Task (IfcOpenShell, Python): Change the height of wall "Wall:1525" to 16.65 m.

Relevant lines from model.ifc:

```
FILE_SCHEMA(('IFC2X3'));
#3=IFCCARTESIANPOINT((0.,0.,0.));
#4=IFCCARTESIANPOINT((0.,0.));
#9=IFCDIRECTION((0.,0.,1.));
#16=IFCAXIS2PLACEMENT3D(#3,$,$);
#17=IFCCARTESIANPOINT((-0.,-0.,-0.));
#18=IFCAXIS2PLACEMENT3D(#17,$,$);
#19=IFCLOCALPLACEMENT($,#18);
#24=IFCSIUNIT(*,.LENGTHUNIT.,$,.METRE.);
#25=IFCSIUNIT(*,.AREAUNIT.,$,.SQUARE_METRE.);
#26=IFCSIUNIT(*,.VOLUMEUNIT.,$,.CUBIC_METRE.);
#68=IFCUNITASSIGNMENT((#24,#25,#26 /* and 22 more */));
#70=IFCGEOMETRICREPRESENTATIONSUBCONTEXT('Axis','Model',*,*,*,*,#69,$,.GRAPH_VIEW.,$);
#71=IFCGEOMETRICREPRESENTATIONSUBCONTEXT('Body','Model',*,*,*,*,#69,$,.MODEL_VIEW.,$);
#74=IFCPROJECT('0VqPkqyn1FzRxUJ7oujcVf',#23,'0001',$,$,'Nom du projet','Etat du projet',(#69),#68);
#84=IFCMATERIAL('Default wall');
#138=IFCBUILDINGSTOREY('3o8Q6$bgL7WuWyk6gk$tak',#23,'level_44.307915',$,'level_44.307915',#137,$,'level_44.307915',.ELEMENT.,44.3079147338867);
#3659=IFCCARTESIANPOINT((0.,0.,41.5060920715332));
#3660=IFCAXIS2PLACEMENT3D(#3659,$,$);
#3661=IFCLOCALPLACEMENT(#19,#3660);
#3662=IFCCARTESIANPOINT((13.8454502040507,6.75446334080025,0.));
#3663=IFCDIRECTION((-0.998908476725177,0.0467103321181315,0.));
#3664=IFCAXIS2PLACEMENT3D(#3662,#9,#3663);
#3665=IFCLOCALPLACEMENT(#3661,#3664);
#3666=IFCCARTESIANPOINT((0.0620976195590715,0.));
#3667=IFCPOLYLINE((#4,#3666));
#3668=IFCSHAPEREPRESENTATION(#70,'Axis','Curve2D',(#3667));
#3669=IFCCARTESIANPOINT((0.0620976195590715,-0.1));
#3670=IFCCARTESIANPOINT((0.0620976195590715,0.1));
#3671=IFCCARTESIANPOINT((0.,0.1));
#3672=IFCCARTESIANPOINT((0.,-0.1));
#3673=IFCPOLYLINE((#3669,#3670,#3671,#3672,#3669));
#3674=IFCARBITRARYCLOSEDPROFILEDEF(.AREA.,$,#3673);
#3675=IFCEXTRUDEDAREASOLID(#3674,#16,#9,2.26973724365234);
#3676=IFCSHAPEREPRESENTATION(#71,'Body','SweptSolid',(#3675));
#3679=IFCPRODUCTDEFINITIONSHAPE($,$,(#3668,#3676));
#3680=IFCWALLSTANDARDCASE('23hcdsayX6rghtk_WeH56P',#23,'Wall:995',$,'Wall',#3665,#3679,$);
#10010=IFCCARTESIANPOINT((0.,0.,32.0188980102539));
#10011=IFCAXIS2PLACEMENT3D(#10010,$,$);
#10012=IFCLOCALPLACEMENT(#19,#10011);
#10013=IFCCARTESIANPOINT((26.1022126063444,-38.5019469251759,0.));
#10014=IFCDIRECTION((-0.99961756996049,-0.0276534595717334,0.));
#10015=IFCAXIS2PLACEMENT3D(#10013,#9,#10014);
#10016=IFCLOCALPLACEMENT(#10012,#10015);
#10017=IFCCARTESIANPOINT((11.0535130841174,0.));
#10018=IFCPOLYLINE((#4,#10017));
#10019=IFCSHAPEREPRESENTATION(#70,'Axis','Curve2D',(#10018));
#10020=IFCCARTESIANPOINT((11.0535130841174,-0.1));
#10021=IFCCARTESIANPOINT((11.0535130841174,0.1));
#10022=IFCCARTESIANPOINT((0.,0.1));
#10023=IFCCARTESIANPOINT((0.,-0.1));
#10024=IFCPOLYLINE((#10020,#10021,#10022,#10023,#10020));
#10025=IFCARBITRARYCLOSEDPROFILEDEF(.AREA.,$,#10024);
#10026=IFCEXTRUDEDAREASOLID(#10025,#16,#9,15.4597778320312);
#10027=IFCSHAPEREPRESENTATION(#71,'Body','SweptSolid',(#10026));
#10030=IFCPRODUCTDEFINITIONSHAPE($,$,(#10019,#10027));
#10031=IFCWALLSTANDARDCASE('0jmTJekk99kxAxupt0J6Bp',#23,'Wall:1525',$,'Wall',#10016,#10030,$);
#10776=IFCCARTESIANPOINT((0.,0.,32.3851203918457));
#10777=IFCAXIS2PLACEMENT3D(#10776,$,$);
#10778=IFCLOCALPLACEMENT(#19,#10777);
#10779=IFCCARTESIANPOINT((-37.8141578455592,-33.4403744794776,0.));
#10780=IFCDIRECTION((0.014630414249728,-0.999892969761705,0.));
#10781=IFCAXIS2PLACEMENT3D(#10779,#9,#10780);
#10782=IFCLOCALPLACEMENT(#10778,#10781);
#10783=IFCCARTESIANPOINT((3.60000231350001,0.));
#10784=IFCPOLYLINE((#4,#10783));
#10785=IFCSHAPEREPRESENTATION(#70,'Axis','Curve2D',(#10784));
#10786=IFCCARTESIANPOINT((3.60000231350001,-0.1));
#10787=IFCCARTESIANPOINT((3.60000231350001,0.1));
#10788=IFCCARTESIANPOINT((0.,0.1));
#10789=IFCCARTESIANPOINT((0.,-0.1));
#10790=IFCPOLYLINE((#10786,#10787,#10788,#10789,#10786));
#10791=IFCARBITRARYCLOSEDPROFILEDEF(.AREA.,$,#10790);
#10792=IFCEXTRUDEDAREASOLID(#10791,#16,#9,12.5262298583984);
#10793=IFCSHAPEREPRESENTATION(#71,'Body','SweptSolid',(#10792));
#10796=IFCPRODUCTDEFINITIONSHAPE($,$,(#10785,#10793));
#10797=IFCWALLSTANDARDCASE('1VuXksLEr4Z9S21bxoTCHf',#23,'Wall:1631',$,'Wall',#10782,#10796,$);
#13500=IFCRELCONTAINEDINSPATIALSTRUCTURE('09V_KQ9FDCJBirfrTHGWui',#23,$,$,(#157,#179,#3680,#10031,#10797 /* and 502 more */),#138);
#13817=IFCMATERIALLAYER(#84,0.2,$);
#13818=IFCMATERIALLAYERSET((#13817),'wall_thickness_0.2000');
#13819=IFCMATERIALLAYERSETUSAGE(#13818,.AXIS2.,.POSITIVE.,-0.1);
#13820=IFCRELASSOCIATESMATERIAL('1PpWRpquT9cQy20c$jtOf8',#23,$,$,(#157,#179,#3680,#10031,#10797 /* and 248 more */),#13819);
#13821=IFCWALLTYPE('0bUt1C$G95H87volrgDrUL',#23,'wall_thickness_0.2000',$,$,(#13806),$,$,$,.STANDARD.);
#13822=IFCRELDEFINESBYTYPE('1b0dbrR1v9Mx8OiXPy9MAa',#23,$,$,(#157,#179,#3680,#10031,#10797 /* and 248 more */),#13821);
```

```python
import ifcopenshell
import ifcopenshell.geom
import ifcopenshell.util.representation
import ifcopenshell.util.shape
import ifcopenshell.util.unit

model = ifcopenshell.open("model.ifc")
unit_scale = ifcopenshell.util.unit.calculate_unit_scale(model)
settings = ifcopenshell.geom.settings()


def volume(element):
    """Net volume in cubic metres, openings subtracted."""
    shape = ifcopenshell.geom.create_shape(settings, element)
    return ifcopenshell.util.shape.get_volume(shape.geometry)


wall = model.by_id(10031)
before = volume(wall)

body = ifcopenshell.util.representation.get_representation(wall, "Model", "Body")
solid = body.Items[0]
old_height = solid.Depth
solid.Depth = 16.65 / unit_scale
after = volume(wall)

print(f"height {old_height:g} -> {solid.Depth:g}, volume {before:.3f} -> {after:.3f} m3")

model.write("model_edited.ifc")
```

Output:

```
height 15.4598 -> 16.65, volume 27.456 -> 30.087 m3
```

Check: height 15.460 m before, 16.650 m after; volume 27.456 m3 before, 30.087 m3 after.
